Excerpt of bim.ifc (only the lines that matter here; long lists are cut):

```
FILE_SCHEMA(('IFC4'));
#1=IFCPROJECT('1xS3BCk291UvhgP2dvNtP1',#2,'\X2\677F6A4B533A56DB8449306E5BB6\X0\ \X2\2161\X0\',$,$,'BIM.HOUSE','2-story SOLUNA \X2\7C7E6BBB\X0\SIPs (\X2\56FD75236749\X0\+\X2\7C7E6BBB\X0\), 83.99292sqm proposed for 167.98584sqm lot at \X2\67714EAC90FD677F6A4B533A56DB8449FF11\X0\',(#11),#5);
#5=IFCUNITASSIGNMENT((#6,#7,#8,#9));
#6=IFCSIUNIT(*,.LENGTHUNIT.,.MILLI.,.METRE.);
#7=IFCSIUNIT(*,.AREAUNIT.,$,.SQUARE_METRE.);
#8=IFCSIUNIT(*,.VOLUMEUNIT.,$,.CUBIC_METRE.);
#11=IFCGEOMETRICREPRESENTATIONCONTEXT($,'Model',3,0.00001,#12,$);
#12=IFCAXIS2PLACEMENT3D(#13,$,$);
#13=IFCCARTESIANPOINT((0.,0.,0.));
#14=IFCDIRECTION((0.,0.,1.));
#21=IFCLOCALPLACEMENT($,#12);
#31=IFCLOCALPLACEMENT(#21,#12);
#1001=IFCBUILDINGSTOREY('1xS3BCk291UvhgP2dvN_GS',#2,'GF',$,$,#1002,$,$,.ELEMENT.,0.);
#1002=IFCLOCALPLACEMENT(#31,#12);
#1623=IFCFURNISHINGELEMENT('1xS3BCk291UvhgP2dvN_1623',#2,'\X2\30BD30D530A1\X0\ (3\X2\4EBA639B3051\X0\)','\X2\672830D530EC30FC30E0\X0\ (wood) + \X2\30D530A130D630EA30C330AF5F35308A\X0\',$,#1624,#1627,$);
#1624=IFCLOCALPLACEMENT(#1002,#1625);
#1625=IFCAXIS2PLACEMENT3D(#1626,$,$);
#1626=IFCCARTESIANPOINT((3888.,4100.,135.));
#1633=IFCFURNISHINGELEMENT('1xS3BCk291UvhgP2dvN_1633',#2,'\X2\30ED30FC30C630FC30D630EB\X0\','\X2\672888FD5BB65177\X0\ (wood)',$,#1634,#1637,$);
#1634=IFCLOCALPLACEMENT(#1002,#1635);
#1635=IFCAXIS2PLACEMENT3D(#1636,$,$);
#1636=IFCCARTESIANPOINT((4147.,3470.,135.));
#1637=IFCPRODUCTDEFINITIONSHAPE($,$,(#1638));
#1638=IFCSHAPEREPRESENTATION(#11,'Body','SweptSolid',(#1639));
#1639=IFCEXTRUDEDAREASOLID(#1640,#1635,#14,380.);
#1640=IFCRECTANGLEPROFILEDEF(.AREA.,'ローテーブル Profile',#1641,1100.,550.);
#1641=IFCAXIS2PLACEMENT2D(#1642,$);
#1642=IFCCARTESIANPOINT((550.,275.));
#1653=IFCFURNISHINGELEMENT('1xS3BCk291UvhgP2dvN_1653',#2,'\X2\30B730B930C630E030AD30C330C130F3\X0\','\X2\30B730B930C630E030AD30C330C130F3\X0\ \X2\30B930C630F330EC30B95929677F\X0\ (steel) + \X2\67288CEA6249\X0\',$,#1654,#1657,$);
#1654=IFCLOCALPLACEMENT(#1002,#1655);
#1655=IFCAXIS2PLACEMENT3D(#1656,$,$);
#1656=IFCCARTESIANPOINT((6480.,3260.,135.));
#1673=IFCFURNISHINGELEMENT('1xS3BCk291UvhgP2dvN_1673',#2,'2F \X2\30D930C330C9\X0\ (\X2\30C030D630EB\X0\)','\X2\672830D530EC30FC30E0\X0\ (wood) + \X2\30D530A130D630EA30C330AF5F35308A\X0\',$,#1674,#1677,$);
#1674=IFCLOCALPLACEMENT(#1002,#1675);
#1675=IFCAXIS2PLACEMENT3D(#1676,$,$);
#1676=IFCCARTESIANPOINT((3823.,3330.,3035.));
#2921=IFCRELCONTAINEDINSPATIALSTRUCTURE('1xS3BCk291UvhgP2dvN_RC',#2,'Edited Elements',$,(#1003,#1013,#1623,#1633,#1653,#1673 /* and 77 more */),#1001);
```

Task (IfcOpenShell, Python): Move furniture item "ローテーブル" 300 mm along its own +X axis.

```python
import ifcopenshell
import ifcopenshell.api.geometry
import ifcopenshell.util.placement

model = ifcopenshell.open("bim.ifc")

item = model.by_id(1633)
matrix = ifcopenshell.util.placement.get_local_placement(item.ObjectPlacement)
matrix[:3, 3] += matrix[:3, 0] * 300.0
ifcopenshell.api.geometry.edit_object_placement(model, product=item, matrix=matrix, is_si=False)

print(ifcopenshell.util.placement.get_local_placement(item.ObjectPlacement).round(3) + 0.0)

model.write("bim_edited.ifc")
```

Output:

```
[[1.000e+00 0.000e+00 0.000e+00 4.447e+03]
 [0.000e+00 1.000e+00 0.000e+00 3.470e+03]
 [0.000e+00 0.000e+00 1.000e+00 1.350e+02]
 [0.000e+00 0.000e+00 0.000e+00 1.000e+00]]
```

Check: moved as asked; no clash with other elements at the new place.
